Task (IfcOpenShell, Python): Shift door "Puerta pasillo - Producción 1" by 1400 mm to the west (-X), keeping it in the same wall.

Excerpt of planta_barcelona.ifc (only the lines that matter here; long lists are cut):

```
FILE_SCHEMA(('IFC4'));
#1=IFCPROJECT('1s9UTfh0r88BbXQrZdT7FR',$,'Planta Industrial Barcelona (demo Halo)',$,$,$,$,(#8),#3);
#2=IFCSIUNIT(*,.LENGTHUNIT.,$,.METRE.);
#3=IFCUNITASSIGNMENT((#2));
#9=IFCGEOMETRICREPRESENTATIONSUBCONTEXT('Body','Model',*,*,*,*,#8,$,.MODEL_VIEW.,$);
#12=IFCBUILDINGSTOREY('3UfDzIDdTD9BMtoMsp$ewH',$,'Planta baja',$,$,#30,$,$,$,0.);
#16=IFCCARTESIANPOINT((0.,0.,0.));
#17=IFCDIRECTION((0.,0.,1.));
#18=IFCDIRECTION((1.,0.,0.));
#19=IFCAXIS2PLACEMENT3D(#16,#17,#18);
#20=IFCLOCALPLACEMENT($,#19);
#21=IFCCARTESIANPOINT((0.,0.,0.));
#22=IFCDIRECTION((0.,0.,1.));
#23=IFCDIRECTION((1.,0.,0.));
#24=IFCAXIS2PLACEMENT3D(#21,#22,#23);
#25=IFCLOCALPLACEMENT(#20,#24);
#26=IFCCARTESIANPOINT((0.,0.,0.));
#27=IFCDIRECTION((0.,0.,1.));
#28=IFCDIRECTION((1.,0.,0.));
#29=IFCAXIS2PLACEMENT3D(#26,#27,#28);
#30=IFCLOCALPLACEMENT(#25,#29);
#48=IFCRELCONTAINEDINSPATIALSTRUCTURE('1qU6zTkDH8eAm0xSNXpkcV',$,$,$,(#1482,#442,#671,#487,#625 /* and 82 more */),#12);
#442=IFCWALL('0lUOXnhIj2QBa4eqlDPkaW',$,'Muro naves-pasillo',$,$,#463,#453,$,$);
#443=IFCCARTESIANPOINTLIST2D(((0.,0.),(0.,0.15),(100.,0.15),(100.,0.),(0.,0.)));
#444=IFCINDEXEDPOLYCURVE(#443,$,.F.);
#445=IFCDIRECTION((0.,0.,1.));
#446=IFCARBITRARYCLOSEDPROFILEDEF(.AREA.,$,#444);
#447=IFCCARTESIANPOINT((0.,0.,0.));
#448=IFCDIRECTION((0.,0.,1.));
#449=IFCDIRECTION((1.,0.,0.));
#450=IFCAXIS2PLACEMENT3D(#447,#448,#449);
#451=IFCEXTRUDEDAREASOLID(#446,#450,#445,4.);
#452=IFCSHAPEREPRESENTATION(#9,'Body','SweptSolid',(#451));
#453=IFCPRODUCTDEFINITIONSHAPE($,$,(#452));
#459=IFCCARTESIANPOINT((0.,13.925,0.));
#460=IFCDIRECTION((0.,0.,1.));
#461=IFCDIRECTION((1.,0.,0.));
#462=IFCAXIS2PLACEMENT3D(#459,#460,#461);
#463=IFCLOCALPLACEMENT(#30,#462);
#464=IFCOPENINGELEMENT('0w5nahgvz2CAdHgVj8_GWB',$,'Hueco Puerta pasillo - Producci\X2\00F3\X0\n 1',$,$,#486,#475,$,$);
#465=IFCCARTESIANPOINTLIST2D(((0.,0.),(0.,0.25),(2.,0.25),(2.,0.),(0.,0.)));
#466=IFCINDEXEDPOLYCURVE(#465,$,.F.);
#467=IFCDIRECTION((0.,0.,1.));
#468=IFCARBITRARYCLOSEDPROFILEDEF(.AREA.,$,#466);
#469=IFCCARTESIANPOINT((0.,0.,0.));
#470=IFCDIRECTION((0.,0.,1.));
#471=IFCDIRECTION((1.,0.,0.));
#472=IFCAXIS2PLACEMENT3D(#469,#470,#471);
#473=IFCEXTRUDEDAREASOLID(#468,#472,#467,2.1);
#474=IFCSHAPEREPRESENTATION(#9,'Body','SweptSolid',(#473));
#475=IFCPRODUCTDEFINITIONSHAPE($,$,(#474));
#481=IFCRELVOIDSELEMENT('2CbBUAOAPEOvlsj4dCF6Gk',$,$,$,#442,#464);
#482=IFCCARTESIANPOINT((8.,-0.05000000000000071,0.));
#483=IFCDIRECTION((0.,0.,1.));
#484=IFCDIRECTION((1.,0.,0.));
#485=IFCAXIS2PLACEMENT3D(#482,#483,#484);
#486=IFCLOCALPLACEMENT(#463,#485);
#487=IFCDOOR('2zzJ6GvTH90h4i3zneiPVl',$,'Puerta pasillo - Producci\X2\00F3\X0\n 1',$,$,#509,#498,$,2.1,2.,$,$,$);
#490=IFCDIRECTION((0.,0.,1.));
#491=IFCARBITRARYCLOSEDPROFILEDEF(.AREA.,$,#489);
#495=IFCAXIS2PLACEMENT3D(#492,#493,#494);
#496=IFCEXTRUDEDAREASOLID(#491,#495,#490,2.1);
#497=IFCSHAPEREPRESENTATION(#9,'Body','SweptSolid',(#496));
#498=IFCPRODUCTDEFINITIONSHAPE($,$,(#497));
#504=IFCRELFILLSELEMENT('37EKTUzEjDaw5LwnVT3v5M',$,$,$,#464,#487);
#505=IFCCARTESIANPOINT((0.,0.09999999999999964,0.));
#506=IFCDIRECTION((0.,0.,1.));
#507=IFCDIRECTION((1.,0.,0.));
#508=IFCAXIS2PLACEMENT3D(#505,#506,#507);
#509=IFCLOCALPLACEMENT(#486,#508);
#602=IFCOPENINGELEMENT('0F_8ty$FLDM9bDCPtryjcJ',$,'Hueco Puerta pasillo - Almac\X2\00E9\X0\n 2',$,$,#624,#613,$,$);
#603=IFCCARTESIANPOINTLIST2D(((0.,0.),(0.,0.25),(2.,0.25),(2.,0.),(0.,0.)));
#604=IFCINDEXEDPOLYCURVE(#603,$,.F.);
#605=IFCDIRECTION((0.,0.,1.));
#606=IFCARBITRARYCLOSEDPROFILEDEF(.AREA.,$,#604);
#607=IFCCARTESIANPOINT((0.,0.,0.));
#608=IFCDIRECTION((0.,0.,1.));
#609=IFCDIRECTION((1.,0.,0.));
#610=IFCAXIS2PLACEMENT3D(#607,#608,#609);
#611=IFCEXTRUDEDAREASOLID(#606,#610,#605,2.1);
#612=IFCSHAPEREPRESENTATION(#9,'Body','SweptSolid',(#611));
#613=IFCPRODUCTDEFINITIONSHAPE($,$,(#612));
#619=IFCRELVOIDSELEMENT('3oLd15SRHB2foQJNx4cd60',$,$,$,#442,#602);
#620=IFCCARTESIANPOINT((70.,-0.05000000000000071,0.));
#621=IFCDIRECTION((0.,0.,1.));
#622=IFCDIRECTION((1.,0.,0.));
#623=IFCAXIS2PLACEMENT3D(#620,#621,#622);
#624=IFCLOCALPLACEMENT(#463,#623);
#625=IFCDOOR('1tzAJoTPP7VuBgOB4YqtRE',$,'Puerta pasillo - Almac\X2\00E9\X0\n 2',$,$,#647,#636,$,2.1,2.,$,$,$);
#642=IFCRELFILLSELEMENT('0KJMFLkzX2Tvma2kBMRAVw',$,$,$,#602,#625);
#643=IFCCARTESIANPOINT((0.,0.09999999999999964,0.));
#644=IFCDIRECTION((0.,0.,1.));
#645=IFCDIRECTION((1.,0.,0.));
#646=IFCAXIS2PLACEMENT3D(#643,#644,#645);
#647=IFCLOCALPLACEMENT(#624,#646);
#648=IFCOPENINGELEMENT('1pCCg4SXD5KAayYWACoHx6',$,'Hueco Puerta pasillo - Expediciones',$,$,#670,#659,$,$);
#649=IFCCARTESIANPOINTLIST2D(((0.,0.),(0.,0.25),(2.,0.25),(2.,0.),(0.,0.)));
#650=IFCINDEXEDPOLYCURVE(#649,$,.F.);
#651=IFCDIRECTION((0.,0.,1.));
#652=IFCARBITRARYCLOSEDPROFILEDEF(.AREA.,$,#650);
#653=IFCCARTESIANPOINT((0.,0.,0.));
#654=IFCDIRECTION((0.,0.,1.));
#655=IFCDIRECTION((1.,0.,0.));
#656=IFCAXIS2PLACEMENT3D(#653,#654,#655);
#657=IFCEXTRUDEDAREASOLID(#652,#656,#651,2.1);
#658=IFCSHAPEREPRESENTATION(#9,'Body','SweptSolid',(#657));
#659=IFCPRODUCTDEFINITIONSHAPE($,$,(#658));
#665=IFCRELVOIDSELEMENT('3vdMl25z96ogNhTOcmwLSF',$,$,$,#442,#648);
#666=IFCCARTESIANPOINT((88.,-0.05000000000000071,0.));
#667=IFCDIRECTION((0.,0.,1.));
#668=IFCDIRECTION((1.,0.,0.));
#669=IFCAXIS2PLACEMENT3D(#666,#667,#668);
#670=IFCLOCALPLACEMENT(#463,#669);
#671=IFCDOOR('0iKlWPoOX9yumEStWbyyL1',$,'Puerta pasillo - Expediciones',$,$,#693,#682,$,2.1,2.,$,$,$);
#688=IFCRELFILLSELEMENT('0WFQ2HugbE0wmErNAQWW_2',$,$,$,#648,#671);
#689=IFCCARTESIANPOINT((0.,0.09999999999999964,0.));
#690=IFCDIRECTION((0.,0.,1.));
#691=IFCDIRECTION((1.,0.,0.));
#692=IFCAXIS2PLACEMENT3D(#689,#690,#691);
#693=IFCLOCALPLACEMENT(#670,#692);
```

```python
import ifcopenshell
import ifcopenshell.api.geometry
import ifcopenshell.util.placement
import ifcopenshell.util.unit

model = ifcopenshell.open("planta_barcelona.ifc")
unit_scale = ifcopenshell.util.unit.calculate_unit_scale(model)

door = model.by_guid("2zzJ6GvTH90h4i3zneiPVl")
opening = door.FillsVoids[0].RelatingOpeningElement
wall = opening.VoidsElements[0].RelatingBuildingElement

wall_matrix = ifcopenshell.util.placement.get_local_placement(wall.ObjectPlacement)
shift = wall_matrix[:3, 0] * -1.4 / unit_scale
before = ifcopenshell.util.placement.get_local_placement(door.ObjectPlacement)[:3, 3].copy()

# The door is placed relative to its opening, so it follows when the opening moves.
matrix = ifcopenshell.util.placement.get_local_placement(opening.ObjectPlacement)
matrix[:3, 3] += shift
ifcopenshell.api.geometry.edit_object_placement(
    model, product=opening, matrix=matrix, is_si=False, should_transform_children=True
)

after = ifcopenshell.util.placement.get_local_placement(door.ObjectPlacement)[:3, 3]
print("door moved by", (after - before).round(3) + 0.0)

model.write("planta_barcelona_updated.ifc")
```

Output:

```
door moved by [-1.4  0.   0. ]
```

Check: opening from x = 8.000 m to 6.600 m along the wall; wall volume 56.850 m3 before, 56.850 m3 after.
